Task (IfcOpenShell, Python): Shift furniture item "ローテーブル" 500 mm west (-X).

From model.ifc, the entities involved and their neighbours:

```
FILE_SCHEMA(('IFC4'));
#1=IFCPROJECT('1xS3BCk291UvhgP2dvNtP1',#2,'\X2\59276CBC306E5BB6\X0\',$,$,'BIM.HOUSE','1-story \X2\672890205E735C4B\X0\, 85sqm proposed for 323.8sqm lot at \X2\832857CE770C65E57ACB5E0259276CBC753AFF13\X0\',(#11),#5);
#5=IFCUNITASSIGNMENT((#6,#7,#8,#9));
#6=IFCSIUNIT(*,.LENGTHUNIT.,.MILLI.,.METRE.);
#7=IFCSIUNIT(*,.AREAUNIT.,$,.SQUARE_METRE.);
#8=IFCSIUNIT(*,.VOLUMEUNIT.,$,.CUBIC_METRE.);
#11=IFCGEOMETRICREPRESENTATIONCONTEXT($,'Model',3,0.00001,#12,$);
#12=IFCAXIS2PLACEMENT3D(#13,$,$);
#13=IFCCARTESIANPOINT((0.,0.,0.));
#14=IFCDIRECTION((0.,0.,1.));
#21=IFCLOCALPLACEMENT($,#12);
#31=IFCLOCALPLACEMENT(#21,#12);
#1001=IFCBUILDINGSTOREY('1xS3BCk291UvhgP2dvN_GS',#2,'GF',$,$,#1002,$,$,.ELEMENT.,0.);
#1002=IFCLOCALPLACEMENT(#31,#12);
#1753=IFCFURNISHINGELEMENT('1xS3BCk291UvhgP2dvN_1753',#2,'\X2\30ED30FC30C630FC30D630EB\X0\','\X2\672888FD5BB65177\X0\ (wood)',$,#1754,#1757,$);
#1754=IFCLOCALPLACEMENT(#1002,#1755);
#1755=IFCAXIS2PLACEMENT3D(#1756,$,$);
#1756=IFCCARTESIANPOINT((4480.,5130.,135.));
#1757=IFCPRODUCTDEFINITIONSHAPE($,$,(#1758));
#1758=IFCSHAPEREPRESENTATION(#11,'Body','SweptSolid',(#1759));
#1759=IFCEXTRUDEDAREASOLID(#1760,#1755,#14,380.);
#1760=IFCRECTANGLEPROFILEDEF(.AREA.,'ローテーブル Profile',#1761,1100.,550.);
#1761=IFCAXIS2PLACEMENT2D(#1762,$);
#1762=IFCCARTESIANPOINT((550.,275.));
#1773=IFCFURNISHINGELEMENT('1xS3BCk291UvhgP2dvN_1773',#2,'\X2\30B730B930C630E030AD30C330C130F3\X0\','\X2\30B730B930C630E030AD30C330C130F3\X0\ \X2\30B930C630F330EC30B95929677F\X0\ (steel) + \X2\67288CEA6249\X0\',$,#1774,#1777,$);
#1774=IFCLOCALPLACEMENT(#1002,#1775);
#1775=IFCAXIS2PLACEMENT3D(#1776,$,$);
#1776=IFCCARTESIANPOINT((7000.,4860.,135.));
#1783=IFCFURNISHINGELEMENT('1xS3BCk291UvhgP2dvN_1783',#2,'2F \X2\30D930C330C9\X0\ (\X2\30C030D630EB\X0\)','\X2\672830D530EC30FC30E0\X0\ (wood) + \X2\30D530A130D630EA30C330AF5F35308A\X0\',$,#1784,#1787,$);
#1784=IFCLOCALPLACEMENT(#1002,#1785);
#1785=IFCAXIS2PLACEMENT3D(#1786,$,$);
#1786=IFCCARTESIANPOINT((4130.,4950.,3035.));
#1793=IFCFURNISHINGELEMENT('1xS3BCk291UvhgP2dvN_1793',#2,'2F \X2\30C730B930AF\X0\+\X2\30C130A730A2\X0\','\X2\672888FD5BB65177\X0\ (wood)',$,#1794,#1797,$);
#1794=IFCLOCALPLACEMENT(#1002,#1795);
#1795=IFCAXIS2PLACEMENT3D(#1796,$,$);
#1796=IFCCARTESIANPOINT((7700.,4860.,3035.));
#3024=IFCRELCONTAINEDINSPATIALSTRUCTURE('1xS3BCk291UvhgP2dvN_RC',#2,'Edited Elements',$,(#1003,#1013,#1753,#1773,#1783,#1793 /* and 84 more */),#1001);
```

```python
import ifcopenshell
import ifcopenshell.api.geometry
import ifcopenshell.util.placement

model = ifcopenshell.open("model.ifc")

item = model.by_id(1753)
matrix = ifcopenshell.util.placement.get_local_placement(item.ObjectPlacement)
matrix[0, 3] -= 500.0
ifcopenshell.api.geometry.edit_object_placement(model, product=item, matrix=matrix, is_si=False)

print(ifcopenshell.util.placement.get_local_placement(item.ObjectPlacement).round(3) + 0.0)

model.write("model_edited.ifc")
```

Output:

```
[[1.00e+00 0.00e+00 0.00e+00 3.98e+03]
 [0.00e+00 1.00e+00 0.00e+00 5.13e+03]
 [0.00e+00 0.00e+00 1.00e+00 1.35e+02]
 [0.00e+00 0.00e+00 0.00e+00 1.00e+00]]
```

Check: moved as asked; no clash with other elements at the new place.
